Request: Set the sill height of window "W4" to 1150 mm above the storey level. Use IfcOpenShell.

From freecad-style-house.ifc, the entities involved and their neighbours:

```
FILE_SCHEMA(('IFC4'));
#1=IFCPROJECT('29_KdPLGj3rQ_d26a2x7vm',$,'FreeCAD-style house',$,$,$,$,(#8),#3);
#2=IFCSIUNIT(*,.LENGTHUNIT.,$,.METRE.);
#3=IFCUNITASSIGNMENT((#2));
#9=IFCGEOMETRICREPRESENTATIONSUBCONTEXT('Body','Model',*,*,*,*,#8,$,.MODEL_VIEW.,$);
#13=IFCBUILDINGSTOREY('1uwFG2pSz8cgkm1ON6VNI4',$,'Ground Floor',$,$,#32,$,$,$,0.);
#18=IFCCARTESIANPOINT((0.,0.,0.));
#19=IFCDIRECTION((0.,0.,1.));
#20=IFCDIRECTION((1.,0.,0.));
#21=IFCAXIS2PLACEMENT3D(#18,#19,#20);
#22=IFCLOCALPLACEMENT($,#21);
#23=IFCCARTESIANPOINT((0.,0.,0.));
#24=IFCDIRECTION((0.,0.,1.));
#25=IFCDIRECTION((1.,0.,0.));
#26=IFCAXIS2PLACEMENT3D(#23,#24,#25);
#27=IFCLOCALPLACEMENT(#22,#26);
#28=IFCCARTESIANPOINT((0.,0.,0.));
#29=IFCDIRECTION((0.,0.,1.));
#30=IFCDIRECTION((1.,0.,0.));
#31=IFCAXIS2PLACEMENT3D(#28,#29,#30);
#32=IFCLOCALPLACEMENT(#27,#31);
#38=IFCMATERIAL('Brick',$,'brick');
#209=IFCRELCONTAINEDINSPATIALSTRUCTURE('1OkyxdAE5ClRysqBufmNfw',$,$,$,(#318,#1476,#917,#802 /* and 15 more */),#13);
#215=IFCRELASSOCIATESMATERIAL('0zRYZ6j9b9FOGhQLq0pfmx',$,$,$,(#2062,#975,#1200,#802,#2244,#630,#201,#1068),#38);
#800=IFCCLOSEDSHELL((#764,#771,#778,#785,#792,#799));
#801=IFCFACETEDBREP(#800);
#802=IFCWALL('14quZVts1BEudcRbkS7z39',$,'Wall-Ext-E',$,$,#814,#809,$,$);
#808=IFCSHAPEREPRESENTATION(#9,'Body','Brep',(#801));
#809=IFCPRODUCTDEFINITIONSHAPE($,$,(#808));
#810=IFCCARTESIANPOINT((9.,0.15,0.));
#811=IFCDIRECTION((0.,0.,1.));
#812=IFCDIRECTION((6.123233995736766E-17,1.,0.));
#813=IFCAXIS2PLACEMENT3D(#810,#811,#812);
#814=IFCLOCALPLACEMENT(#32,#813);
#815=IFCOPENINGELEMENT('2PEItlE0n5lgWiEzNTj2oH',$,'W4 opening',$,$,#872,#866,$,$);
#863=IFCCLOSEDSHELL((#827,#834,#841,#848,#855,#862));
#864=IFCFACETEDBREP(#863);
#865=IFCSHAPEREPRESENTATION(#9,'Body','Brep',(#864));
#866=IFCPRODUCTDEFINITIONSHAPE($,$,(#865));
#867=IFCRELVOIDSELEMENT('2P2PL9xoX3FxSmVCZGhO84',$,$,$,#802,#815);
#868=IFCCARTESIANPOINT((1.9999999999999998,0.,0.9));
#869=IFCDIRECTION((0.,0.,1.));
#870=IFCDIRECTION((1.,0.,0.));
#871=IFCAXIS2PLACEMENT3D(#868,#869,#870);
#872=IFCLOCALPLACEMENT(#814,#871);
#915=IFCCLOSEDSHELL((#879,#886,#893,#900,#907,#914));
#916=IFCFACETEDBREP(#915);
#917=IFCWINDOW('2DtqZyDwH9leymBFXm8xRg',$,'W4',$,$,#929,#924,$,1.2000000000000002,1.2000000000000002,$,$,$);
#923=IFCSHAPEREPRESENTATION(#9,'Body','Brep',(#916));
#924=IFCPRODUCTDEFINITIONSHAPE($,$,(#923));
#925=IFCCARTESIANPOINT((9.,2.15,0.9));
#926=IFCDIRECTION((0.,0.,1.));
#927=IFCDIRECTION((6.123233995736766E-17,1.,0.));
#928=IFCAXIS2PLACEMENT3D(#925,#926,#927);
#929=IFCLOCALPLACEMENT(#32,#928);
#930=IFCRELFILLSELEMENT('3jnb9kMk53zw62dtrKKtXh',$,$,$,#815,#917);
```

```python
import numpy as np
import ifcopenshell
import ifcopenshell.api.geometry
import ifcopenshell.geom
import ifcopenshell.util.element
import ifcopenshell.util.placement
import ifcopenshell.util.shape
import ifcopenshell.util.unit

model = ifcopenshell.open("freecad-style-house.ifc")
unit_scale = ifcopenshell.util.unit.calculate_unit_scale(model)

window = model.by_guid("2DtqZyDwH9leymBFXm8xRg")
opening = window.FillsVoids[0].RelatingOpeningElement
storey = ifcopenshell.util.element.get_container(window, ifc_class="IfcBuildingStorey")
level = ifcopenshell.util.placement.get_local_placement(storey.ObjectPlacement)[2, 3]

# The opening's origin need not be at the sill, so measure its lowest point.
shape = ifcopenshell.geom.create_shape(ifcopenshell.geom.settings(), opening)
bottom = ifcopenshell.util.shape.get_shape_bottom_elevation(shape, shape.geometry) / unit_scale
dz = level + 1.15 / unit_scale - bottom

shift = np.array([0.0, 0.0, dz])
# The window is not placed relative to its opening, so move both.
for product in (opening, window):
    matrix = ifcopenshell.util.placement.get_local_placement(product.ObjectPlacement)
    matrix[:3, 3] += shift
    ifcopenshell.api.geometry.edit_object_placement(model, product=product, matrix=matrix, is_si=False)

print(f"moved by {dz * unit_scale:+.3f} m")

model.write("freecad-style-house_edited.ifc")
```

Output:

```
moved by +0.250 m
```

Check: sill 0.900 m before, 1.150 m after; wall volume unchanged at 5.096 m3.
